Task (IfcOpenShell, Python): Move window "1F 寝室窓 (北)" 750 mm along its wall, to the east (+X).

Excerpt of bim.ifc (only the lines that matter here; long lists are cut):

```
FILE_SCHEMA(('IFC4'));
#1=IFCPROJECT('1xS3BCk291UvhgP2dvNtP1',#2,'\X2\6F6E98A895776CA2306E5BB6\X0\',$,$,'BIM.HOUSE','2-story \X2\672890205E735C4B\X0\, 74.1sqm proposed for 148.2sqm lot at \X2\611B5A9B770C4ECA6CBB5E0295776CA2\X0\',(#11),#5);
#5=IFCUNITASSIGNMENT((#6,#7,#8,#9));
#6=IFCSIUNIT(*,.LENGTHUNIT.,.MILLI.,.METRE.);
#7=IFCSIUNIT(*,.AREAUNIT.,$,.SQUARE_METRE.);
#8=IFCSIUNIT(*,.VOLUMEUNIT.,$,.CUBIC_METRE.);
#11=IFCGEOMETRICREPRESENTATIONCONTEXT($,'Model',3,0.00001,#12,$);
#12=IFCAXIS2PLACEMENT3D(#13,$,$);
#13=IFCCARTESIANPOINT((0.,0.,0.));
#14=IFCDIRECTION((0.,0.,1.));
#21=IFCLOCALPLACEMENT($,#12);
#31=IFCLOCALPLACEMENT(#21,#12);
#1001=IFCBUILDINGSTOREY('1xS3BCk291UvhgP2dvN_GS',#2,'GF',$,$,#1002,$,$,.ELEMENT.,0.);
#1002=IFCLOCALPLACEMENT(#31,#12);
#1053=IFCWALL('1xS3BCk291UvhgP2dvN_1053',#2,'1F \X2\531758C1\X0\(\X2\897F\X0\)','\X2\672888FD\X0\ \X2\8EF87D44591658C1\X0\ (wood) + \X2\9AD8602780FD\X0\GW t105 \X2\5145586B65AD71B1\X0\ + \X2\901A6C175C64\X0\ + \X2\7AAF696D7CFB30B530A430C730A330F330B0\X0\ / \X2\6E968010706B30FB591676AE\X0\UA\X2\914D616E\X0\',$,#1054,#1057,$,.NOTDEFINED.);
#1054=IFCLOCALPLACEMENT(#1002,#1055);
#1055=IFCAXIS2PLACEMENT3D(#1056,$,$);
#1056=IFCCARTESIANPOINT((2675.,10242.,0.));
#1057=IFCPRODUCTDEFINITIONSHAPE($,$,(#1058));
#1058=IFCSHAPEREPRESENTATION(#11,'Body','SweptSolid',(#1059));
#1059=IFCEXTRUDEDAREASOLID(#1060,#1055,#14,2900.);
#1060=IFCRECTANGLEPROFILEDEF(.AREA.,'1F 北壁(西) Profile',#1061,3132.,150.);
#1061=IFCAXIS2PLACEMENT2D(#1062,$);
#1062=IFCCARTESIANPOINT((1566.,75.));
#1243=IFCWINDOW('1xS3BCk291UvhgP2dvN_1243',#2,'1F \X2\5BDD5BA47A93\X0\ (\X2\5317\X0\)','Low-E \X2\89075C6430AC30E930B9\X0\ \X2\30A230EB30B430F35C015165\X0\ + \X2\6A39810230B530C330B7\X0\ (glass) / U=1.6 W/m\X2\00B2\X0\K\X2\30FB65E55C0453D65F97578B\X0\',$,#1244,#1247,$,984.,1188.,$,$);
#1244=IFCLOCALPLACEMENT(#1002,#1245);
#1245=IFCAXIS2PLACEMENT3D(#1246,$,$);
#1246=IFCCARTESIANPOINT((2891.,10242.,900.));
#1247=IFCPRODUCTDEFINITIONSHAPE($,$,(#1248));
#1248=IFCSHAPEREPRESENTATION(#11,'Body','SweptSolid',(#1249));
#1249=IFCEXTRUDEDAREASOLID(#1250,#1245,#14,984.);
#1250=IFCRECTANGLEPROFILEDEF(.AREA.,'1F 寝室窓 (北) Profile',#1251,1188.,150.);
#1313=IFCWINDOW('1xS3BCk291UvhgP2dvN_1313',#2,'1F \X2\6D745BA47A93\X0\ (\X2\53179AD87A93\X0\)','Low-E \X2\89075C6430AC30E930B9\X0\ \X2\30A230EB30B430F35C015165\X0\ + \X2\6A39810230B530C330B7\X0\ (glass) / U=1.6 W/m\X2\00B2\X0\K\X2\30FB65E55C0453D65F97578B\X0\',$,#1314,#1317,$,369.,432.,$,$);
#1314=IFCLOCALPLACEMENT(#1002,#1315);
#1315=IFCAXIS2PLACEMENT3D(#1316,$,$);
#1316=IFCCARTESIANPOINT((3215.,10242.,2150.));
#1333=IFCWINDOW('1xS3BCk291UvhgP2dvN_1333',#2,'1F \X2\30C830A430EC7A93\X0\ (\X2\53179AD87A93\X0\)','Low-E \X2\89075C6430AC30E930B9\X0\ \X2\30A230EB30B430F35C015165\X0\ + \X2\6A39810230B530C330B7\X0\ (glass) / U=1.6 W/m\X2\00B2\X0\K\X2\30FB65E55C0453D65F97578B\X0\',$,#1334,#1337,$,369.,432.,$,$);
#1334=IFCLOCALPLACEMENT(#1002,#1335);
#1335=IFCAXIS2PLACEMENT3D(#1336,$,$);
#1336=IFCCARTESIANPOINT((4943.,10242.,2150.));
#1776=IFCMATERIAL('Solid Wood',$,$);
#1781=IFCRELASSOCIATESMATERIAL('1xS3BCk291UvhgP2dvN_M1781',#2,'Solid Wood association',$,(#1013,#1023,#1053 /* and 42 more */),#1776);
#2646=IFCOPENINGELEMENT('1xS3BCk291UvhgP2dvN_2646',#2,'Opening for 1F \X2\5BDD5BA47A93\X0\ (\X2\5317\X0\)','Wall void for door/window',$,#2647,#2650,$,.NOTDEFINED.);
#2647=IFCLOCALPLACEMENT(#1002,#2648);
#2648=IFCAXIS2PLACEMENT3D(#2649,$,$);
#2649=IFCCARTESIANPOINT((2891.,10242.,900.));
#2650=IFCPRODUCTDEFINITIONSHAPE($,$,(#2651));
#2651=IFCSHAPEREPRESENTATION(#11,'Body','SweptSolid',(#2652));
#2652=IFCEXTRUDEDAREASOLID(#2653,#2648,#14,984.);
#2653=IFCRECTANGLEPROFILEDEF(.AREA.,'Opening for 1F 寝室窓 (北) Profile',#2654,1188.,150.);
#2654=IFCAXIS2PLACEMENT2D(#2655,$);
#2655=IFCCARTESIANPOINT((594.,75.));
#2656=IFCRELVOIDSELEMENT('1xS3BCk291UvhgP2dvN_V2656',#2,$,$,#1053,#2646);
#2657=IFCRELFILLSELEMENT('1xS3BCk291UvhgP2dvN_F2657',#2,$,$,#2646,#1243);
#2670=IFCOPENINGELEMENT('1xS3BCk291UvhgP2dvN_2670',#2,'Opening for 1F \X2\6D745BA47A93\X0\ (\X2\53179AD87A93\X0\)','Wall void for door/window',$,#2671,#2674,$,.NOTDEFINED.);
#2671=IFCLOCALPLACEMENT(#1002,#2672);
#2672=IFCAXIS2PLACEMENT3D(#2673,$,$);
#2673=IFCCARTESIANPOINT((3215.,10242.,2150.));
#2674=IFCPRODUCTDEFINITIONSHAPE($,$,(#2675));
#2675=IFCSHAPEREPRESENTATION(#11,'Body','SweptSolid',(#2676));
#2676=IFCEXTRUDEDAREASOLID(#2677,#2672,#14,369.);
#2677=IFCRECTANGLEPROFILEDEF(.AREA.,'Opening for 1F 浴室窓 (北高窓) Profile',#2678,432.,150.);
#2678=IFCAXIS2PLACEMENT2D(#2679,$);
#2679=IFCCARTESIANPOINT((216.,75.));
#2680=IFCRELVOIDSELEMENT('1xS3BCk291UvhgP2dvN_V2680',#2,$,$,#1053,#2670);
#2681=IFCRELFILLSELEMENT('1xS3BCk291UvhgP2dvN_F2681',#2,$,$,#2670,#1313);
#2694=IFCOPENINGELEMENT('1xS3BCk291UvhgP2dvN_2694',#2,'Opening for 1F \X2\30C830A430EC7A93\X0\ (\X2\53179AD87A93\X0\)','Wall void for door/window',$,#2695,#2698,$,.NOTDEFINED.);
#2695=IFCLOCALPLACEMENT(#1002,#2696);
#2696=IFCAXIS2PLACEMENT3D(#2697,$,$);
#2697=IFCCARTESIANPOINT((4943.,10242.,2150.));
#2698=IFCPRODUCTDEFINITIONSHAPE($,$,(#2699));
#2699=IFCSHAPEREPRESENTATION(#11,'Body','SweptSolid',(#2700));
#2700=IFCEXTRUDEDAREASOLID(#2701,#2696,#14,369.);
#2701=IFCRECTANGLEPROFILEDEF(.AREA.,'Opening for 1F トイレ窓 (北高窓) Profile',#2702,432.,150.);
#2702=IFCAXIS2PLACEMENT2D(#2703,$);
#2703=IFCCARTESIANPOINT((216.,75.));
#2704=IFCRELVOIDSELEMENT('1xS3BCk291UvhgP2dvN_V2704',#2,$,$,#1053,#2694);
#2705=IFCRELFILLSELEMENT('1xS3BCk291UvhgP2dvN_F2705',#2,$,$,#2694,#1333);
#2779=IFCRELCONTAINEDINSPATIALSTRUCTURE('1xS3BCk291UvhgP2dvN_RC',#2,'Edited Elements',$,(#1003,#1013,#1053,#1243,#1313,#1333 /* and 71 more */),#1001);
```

```python
import ifcopenshell
import ifcopenshell.api.geometry
import ifcopenshell.util.placement
import ifcopenshell.util.unit

model = ifcopenshell.open("bim.ifc")
unit_scale = ifcopenshell.util.unit.calculate_unit_scale(model)

window = model.by_guid("1xS3BCk291UvhgP2dvN_1243")
opening = window.FillsVoids[0].RelatingOpeningElement
wall = opening.VoidsElements[0].RelatingBuildingElement

wall_matrix = ifcopenshell.util.placement.get_local_placement(wall.ObjectPlacement)
shift = wall_matrix[:3, 0] * 0.75 / unit_scale
before = ifcopenshell.util.placement.get_local_placement(window.ObjectPlacement)[:3, 3].copy()

# The window is not placed relative to its opening, so move both.
for product in (opening, window):
    matrix = ifcopenshell.util.placement.get_local_placement(product.ObjectPlacement)
    matrix[:3, 3] += shift
    ifcopenshell.api.geometry.edit_object_placement(model, product=product, matrix=matrix, is_si=False)

after = ifcopenshell.util.placement.get_local_placement(window.ObjectPlacement)[:3, 3]
print("window moved by", (after - before).round(3) + 0.0)

model.write("bim_edited.ifc")
```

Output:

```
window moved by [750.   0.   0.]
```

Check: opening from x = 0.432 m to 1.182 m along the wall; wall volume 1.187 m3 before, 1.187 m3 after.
